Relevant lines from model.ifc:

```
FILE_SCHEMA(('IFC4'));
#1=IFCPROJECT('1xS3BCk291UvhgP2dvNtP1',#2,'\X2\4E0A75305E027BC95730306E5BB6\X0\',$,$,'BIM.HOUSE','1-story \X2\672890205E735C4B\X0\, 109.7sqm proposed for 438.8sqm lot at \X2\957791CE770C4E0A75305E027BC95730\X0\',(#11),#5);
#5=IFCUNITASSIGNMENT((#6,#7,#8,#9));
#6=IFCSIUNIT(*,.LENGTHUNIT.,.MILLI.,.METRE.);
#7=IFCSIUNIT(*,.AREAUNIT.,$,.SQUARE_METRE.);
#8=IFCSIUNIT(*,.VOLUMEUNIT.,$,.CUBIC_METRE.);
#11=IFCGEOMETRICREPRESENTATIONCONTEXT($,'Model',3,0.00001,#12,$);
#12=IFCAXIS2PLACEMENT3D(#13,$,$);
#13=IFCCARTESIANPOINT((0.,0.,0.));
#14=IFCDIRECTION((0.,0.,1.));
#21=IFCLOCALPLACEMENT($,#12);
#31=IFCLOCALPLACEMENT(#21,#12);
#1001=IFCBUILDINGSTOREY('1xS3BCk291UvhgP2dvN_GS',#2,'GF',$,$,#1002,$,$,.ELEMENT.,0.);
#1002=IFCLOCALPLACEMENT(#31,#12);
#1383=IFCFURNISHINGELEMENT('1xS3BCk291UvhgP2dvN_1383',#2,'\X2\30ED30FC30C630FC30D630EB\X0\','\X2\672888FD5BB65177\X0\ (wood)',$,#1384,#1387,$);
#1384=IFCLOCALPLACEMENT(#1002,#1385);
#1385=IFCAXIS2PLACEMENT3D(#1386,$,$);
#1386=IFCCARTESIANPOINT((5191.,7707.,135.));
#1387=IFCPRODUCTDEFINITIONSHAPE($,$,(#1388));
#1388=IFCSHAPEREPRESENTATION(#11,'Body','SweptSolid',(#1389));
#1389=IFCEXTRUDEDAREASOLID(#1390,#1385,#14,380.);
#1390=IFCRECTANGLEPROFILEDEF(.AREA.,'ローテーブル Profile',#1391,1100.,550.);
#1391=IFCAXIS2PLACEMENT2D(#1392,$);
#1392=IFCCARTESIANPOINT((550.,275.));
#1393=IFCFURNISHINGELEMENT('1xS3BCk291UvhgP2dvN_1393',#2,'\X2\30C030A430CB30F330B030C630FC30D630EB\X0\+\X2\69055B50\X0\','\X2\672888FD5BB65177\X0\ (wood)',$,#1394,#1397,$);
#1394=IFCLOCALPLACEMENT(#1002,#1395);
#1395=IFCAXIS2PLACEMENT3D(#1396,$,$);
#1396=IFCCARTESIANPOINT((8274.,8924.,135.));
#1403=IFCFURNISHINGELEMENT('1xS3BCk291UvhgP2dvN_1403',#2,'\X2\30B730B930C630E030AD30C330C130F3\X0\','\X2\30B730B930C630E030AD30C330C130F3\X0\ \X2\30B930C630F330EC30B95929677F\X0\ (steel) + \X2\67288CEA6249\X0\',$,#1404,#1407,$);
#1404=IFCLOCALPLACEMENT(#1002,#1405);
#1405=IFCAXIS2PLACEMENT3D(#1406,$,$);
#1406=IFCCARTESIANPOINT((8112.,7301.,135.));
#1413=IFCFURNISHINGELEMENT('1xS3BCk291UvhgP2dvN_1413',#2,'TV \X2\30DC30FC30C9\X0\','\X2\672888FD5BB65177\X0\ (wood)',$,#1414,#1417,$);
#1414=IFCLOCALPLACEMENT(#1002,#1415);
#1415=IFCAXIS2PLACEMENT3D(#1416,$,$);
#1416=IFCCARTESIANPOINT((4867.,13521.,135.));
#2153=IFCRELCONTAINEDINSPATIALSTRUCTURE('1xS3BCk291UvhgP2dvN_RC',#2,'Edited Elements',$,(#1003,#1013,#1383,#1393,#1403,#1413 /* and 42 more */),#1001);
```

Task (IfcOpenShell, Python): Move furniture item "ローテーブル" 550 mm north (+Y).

```python
import ifcopenshell
import ifcopenshell.api.geometry
import ifcopenshell.util.placement
import ifcopenshell.util.unit

model = ifcopenshell.open("model.ifc")
unit_scale = ifcopenshell.util.unit.calculate_unit_scale(model)

item = model.by_guid("1xS3BCk291UvhgP2dvN_1383")
matrix = ifcopenshell.util.placement.get_local_placement(item.ObjectPlacement)
matrix[1, 3] += 0.55 / unit_scale
ifcopenshell.api.geometry.edit_object_placement(model, product=item, matrix=matrix, is_si=False)

print(ifcopenshell.util.placement.get_local_placement(item.ObjectPlacement).round(3) + 0.0)

model.write("model_updated.ifc")
```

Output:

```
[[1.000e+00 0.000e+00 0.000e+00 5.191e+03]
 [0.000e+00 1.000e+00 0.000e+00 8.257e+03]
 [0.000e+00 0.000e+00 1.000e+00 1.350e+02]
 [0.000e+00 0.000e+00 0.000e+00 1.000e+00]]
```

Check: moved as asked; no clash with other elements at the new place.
